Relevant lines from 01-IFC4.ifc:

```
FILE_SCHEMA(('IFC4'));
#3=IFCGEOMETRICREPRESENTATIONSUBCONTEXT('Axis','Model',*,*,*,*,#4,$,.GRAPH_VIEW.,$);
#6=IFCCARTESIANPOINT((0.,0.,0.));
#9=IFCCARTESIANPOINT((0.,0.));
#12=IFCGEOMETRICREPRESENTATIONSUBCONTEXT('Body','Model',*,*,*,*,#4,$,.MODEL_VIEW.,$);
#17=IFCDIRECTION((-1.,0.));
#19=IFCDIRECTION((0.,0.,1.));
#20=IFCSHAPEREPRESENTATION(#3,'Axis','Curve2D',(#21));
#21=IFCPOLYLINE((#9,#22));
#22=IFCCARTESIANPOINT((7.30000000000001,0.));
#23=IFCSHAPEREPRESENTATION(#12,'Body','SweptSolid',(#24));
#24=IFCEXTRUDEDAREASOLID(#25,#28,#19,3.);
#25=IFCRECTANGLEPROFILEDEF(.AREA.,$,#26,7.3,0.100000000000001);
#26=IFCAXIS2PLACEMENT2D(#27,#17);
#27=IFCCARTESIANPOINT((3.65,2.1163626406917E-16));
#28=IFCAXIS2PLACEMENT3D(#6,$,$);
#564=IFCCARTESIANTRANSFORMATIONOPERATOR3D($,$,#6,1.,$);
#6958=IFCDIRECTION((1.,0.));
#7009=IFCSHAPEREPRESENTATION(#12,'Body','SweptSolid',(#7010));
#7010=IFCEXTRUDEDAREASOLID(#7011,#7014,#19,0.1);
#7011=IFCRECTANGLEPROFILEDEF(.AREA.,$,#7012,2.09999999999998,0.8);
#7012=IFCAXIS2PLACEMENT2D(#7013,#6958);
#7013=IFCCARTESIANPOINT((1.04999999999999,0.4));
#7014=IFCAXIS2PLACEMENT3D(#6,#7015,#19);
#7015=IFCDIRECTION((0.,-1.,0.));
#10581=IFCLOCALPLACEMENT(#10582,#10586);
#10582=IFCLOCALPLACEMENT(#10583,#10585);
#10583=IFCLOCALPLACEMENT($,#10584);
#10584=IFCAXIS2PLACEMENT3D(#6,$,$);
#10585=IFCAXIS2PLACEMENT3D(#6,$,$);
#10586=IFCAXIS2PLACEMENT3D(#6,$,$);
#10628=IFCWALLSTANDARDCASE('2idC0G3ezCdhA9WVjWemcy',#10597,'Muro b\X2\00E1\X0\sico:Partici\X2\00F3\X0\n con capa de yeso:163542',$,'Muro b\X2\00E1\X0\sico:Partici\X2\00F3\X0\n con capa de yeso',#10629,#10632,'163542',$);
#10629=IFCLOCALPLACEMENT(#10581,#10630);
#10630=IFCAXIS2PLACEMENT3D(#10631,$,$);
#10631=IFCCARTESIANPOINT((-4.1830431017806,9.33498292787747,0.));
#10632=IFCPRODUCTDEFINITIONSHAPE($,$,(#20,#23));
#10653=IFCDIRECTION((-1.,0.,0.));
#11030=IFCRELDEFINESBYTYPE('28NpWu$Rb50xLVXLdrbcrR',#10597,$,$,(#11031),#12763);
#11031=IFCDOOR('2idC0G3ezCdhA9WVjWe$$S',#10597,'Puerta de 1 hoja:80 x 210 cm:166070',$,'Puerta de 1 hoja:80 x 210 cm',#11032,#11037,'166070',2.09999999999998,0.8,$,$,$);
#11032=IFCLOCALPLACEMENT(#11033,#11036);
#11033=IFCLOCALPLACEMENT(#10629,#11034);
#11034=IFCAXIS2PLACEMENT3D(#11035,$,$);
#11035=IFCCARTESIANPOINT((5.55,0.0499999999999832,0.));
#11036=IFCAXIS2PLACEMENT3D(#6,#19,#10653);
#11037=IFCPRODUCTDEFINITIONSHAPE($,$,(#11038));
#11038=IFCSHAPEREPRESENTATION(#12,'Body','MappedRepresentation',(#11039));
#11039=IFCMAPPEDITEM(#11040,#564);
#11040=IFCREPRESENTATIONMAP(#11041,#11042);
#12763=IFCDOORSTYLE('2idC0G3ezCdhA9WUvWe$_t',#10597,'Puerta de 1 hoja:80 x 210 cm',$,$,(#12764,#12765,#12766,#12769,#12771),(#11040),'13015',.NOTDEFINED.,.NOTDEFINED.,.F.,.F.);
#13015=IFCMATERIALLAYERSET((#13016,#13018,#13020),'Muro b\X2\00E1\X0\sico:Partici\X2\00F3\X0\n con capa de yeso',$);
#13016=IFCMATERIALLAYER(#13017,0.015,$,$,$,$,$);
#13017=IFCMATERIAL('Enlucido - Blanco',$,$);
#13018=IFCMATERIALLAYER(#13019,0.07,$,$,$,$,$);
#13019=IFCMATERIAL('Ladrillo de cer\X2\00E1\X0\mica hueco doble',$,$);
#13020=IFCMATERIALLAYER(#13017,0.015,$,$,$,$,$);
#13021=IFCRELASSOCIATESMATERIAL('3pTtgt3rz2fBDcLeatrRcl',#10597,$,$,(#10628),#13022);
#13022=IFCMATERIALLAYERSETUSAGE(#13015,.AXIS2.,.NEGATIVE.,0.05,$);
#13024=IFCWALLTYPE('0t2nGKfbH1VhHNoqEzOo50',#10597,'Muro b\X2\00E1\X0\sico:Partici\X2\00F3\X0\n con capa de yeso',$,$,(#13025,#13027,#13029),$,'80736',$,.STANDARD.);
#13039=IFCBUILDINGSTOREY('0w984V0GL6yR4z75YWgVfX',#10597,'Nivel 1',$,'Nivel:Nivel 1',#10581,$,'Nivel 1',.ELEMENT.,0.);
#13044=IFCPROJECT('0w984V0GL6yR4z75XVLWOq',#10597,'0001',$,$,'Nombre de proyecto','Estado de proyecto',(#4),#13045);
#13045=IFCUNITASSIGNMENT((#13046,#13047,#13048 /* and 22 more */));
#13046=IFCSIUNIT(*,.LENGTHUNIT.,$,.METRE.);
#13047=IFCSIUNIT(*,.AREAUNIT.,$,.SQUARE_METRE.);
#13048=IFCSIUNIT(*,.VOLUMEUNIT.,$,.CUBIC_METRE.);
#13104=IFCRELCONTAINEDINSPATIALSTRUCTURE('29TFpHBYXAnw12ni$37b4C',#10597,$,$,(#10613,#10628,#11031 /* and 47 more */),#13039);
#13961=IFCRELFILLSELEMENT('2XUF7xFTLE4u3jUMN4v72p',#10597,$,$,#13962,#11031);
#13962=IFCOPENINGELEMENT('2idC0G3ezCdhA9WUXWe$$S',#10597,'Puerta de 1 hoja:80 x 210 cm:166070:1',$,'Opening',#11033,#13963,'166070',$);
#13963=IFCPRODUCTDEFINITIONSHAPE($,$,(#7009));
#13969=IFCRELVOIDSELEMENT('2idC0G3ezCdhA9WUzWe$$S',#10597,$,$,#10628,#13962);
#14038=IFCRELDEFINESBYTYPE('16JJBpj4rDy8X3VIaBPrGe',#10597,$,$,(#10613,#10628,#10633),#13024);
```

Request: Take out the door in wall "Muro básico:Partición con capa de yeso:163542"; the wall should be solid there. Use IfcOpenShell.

```python
import ifcopenshell
import ifcopenshell.api.feature
import ifcopenshell.api.root
import ifcopenshell.geom
import ifcopenshell.util.shape

model = ifcopenshell.open("01-IFC4.ifc")
settings = ifcopenshell.geom.settings()


def volume(element):
    """Net volume in cubic metres, openings subtracted."""
    shape = ifcopenshell.geom.create_shape(settings, element)
    return ifcopenshell.util.shape.get_volume(shape.geometry)


door = model.by_guid("2idC0G3ezCdhA9WVjWe$$S")
opening = door.FillsVoids[0].RelatingOpeningElement
wall = opening.VoidsElements[0].RelatingBuildingElement
before = volume(wall)

ifcopenshell.api.root.remove_product(model, product=door)
ifcopenshell.api.feature.remove_feature(model, feature=opening)

after = volume(wall)

print(f"wall volume {before:.3f} -> {after:.3f} m3")

model.write("01-IFC4-out.ifc")
```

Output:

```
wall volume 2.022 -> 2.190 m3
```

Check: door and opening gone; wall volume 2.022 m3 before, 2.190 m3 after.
